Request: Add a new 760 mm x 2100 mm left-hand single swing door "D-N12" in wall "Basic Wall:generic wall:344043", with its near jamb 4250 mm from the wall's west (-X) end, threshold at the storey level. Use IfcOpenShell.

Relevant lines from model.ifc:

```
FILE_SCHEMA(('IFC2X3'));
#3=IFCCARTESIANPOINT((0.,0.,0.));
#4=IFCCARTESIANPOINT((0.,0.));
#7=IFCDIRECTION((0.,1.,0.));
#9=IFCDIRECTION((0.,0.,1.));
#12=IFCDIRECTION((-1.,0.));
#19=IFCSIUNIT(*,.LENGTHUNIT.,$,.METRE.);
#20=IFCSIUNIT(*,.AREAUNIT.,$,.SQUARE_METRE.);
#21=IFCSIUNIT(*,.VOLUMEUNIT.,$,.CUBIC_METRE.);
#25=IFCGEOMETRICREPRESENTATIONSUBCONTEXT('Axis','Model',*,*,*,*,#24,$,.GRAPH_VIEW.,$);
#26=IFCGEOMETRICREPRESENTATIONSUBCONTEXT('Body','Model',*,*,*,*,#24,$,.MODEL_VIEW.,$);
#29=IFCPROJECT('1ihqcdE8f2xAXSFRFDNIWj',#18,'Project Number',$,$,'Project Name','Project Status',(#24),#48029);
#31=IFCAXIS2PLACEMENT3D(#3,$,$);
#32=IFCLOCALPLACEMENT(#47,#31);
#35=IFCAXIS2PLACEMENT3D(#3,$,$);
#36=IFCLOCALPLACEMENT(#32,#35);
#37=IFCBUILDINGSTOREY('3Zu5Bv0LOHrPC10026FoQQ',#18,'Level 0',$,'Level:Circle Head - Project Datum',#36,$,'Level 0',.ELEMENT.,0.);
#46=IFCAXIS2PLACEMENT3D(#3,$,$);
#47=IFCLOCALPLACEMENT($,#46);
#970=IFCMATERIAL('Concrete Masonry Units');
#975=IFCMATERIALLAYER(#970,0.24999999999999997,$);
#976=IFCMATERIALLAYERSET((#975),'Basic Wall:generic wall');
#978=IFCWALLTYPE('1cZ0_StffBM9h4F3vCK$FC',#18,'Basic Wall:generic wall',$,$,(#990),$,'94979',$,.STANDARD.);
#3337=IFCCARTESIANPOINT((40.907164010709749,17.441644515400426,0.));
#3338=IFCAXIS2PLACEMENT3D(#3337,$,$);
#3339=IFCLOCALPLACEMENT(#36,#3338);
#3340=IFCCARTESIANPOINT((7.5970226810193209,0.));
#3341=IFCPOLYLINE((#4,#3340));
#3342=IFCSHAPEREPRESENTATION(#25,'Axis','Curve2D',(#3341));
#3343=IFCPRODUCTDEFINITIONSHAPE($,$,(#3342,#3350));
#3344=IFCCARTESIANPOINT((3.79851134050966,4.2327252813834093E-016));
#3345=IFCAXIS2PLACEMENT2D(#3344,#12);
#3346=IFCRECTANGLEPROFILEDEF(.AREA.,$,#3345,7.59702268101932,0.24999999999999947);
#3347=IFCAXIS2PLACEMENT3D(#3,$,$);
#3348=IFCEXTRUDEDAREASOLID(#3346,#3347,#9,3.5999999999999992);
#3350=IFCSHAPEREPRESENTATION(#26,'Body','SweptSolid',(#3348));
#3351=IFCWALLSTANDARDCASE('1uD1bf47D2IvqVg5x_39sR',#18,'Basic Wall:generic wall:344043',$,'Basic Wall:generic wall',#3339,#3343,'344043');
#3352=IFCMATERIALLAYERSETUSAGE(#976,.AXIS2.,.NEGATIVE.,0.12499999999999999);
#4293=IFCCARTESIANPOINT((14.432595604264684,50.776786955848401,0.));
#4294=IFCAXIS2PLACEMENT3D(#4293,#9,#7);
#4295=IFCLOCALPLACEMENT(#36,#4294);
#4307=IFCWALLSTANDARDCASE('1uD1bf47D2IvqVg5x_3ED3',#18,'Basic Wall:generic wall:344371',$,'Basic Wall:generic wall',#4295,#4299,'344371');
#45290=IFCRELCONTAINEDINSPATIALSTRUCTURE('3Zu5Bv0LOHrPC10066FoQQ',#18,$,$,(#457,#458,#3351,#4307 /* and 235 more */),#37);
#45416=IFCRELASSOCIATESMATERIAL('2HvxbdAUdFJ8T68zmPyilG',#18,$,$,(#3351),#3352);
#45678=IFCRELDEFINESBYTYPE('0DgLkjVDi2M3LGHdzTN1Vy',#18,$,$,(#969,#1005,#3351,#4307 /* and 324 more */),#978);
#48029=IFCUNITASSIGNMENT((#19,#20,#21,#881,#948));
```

```python
import numpy as np
import ifcopenshell
import ifcopenshell.api.feature
import ifcopenshell.api.geometry
import ifcopenshell.api.root
import ifcopenshell.api.spatial
import ifcopenshell.api.type
import ifcopenshell.geom
import ifcopenshell.util.element
import ifcopenshell.util.placement
import ifcopenshell.util.representation
import ifcopenshell.util.shape
import ifcopenshell.util.unit

model = ifcopenshell.open("model.ifc")
unit_scale = ifcopenshell.util.unit.calculate_unit_scale(model)
settings = ifcopenshell.geom.settings()


def volume(element):
    """Net volume in cubic metres, openings subtracted."""
    shape = ifcopenshell.geom.create_shape(settings, element)
    return ifcopenshell.util.shape.get_volume(shape.geometry)


wall = model.by_guid("1uD1bf47D2IvqVg5x_39sR")
storey = ifcopenshell.util.element.get_container(wall, ifc_class="IfcBuildingStorey")
context = ifcopenshell.util.representation.get_context(model, "Model", "Body", "MODEL_VIEW")
before = volume(wall)

width, height, from_end, sill = 0.76, 2.1, 4.25, 0.0  # metres

# The wall runs along its own X axis, and the end named is its -X end.
wall_shape = ifcopenshell.geom.create_shape(settings, wall)
x, y, z = ifcopenshell.util.shape.get_vertices(wall_shape.geometry).T
start = x.min() + from_end
face, thickness = float(y.min()), float(y.max() - y.min())
wall_matrix = ifcopenshell.util.placement.get_local_placement(wall.ObjectPlacement)
level = ifcopenshell.util.placement.get_local_placement(storey.ObjectPlacement)[2, 3]


def in_wall(x, y):
    """Placement at x, y metres in the wall's axes, at sill height."""
    matrix = wall_matrix.copy()
    matrix[:, 3] = wall_matrix @ np.array([x / unit_scale, y / unit_scale, 0.0, 1.0])
    matrix[2, 3] = level + sill / unit_scale
    return matrix


# Opening: a box that overshoots both wall faces by 50 mm.
opening = ifcopenshell.api.root.create_entity(model, ifc_class="IfcOpeningElement")
box = ifcopenshell.api.geometry.add_wall_representation(
    model, context=context, length=width, height=height, thickness=thickness + 0.1
)
ifcopenshell.api.geometry.assign_representation(model, product=opening, representation=box)
ifcopenshell.api.geometry.edit_object_placement(model, product=opening, matrix=in_wall(start, face - 0.05), is_si=False)
ifcopenshell.api.feature.add_feature(model, feature=opening, element=wall)

door = ifcopenshell.api.root.create_entity(model, ifc_class="IfcDoor", name="D-N12")
door.OverallWidth, door.OverallHeight = width / unit_scale, height / unit_scale
body = ifcopenshell.api.geometry.add_door_representation(
    model,
    context=context,
    overall_width=door.OverallWidth,
    overall_height=door.OverallHeight,
    operation_type="SINGLE_SWING_LEFT",
    lining_properties={"LiningDepth": thickness / unit_scale, "ThresholdDepth": thickness / unit_scale},
)
ifcopenshell.api.geometry.assign_representation(model, product=door, representation=body)
ifcopenshell.api.spatial.assign_container(model, products=[door], relating_structure=storey)
fills = ifcopenshell.api.feature.add_filling(model, opening=opening, element=door)
fills.OwnerHistory = door.OwnerHistory  # required in IFC2X3

# IFC2X3 keeps the operation on the door style.
style = ifcopenshell.api.root.create_entity(model, ifc_class="IfcDoorStyle", name="D-N12")
style.OperationType, style.ConstructionType = "SINGLE_SWING_LEFT", "NOTDEFINED"
style.ParameterTakesPrecedence = style.Sizeable = False
ifcopenshell.api.type.assign_type(model, related_objects=[door], relating_type=style)

# The lining spans the wall, so the door starts at the wall face.
ifcopenshell.api.geometry.edit_object_placement(model, product=door, matrix=in_wall(start, face), is_si=False)

after = volume(wall)

print(f"wall volume {before:.3f} -> {after:.3f} m3")

model.write("model_v2.ifc")
```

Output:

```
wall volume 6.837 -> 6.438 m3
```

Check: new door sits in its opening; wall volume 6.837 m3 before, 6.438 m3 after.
